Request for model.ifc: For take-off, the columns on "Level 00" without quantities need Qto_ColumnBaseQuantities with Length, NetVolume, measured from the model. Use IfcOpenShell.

First a look at what the model holds.

```python
import ifcopenshell
import ifcopenshell.util.element
import ifcopenshell.util.unit

model = ifcopenshell.open("model.ifc")
print(model.schema)
for unit_type in ("LENGTHUNIT", "AREAUNIT", "VOLUMEUNIT"):
    print(unit_type, ifcopenshell.util.unit.calculate_unit_scale(model, unit_type))
storey = next(s for s in model.by_type("IfcBuildingStorey") if s.Name == "Level 00")
columns = [e for e in ifcopenshell.util.element.get_decomposition(storey) if e.is_a("IfcColumn")]
for e in sorted(columns, key=lambda e: e.id()):
    print(e.id(), e.is_a(), e.Name, list(ifcopenshell.util.element.get_psets(e, qtos_only=True)), sep=" | ")
```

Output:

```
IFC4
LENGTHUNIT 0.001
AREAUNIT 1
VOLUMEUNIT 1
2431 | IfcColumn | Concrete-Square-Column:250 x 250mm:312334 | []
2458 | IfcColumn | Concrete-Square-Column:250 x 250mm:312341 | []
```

```python
import ifcopenshell
import ifcopenshell.api.pset
import ifcopenshell.geom
import ifcopenshell.util.element
import ifcopenshell.util.shape
import ifcopenshell.util.unit

model = ifcopenshell.open("model.ifc")
unit_scale = ifcopenshell.util.unit.calculate_unit_scale(model)
volume_scale = ifcopenshell.util.unit.calculate_unit_scale(model, "VOLUMEUNIT")
settings = ifcopenshell.geom.settings()

storey = next(s for s in model.by_type("IfcBuildingStorey") if s.Name == "Level 00")
columns = [e for e in ifcopenshell.util.element.get_decomposition(storey) if e.is_a("IfcColumn")]

for e in sorted(columns, key=lambda e: e.id()):
    if ifcopenshell.util.element.get_psets(e, qtos_only=True, should_inherit=False):
        continue
    # Geometry comes back in metres, in the element's own axes.
    shape = ifcopenshell.geom.create_shape(settings, e)
    values = {
        "Length": ifcopenshell.util.shape.get_z(shape.geometry) / unit_scale,
        "NetVolume": ifcopenshell.util.shape.get_volume(shape.geometry) / volume_scale,
    }
    qto = ifcopenshell.api.pset.add_qto(model, product=e, name="Qto_ColumnBaseQuantities")
    ifcopenshell.api.pset.edit_qto(model, qto=qto, properties=values)
    print(e.id(), {k: round(v, 3) for k, v in values.items()})

model.write("model-out.ifc")
```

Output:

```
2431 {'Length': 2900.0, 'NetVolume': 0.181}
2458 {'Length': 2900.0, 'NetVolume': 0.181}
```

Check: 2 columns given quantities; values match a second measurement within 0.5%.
